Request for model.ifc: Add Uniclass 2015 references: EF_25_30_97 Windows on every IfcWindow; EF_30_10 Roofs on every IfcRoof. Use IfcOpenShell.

First a look at what the model holds.

```python
import ifcopenshell

model = ifcopenshell.open("model.ifc")
print(model.schema)
print("classifications:", [c.Name for c in model.by_type("IfcClassification")])
for ifc_class in ("IfcDoor", "IfcRoof", "IfcStair", "IfcWall", "IfcWindow"):
    print(ifc_class, len(model.by_type(ifc_class)))
```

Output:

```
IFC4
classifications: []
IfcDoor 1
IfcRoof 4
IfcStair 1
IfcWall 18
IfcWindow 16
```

```python
import ifcopenshell
import ifcopenshell.api.classification

model = ifcopenshell.open("model.ifc")

system = ifcopenshell.api.classification.add_classification(model, classification="Uniclass 2015")

codes = {
    "IfcWindow": ("EF_25_30_97", "Windows"),
    "IfcRoof": ("EF_30_10", "Roofs"),
}
for ifc_class, (code, name) in codes.items():
    products = model.by_type(ifc_class)
    ifcopenshell.api.classification.add_reference(
        model, products=products, classification=system, identification=code, name=name
    )
    print(code, len(products))

model.write("model_v2.ifc")
```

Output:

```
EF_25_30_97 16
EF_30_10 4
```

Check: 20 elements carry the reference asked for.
